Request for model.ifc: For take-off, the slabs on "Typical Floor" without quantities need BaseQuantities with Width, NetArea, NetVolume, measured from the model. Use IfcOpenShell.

First a look at what the model holds.

```python
import ifcopenshell
import ifcopenshell.util.element
import ifcopenshell.util.unit

model = ifcopenshell.open("model.ifc")
print(model.schema)
for unit_type in ("LENGTHUNIT", "AREAUNIT", "VOLUMEUNIT"):
    print(unit_type, ifcopenshell.util.unit.calculate_unit_scale(model, unit_type))
storey = next(s for s in model.by_type("IfcBuildingStorey") if s.Name == "Typical Floor")
slabs = [e for e in ifcopenshell.util.element.get_decomposition(storey) if e.is_a("IfcSlab")]
for e in sorted(slabs, key=lambda e: e.id()):
    print(e.id(), e.is_a(), e.Name, list(ifcopenshell.util.element.get_psets(e, qtos_only=True)), sep=" | ")
```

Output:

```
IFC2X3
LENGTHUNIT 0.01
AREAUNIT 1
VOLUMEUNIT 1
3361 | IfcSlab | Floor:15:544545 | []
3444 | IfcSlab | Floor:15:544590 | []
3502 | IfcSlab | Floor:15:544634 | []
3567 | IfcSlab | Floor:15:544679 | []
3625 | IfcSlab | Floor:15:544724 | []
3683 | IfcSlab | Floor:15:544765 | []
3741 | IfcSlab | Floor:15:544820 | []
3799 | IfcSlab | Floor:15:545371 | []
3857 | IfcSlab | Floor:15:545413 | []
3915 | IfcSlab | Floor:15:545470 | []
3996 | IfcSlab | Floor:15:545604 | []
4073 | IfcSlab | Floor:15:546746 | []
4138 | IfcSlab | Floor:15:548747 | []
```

```python
import ifcopenshell
import ifcopenshell.api.pset
import ifcopenshell.geom
import ifcopenshell.util.element
import ifcopenshell.util.shape
import ifcopenshell.util.unit

model = ifcopenshell.open("model.ifc")
unit_scale = ifcopenshell.util.unit.calculate_unit_scale(model)
area_scale = ifcopenshell.util.unit.calculate_unit_scale(model, "AREAUNIT")
volume_scale = ifcopenshell.util.unit.calculate_unit_scale(model, "VOLUMEUNIT")
settings = ifcopenshell.geom.settings()

storey = next(s for s in model.by_type("IfcBuildingStorey") if s.Name == "Typical Floor")
slabs = [e for e in ifcopenshell.util.element.get_decomposition(storey) if e.is_a("IfcSlab")]

for e in sorted(slabs, key=lambda e: e.id()):
    if ifcopenshell.util.element.get_psets(e, qtos_only=True, should_inherit=False):
        continue
    # Geometry comes back in metres, in the element's own axes.
    shape = ifcopenshell.geom.create_shape(settings, e)
    values = {
        "Width": ifcopenshell.util.shape.get_z(shape.geometry) / unit_scale,
        "NetArea": ifcopenshell.util.shape.get_footprint_area(shape.geometry) / area_scale,
        "NetVolume": ifcopenshell.util.shape.get_volume(shape.geometry) / volume_scale,
    }
    qto = ifcopenshell.api.pset.add_qto(model, product=e, name="BaseQuantities")
    ifcopenshell.api.pset.edit_qto(model, qto=qto, properties=values)
    print(e.id(), {k: round(v, 3) for k, v in values.items()})

model.write("model_v2.ifc")
```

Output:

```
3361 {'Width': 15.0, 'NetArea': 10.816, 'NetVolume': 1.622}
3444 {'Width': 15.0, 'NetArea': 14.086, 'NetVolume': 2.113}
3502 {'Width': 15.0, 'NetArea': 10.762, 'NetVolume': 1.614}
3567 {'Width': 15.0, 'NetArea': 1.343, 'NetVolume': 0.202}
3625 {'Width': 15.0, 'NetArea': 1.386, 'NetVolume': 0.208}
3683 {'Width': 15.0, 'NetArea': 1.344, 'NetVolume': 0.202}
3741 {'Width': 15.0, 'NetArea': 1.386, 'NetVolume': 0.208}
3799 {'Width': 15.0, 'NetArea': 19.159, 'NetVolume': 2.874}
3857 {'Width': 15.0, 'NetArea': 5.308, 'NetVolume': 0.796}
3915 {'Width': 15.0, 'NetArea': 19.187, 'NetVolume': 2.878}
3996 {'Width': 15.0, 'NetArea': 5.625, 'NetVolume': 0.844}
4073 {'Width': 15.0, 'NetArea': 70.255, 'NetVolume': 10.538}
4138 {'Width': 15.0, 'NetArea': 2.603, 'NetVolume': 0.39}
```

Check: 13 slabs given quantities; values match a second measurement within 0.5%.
